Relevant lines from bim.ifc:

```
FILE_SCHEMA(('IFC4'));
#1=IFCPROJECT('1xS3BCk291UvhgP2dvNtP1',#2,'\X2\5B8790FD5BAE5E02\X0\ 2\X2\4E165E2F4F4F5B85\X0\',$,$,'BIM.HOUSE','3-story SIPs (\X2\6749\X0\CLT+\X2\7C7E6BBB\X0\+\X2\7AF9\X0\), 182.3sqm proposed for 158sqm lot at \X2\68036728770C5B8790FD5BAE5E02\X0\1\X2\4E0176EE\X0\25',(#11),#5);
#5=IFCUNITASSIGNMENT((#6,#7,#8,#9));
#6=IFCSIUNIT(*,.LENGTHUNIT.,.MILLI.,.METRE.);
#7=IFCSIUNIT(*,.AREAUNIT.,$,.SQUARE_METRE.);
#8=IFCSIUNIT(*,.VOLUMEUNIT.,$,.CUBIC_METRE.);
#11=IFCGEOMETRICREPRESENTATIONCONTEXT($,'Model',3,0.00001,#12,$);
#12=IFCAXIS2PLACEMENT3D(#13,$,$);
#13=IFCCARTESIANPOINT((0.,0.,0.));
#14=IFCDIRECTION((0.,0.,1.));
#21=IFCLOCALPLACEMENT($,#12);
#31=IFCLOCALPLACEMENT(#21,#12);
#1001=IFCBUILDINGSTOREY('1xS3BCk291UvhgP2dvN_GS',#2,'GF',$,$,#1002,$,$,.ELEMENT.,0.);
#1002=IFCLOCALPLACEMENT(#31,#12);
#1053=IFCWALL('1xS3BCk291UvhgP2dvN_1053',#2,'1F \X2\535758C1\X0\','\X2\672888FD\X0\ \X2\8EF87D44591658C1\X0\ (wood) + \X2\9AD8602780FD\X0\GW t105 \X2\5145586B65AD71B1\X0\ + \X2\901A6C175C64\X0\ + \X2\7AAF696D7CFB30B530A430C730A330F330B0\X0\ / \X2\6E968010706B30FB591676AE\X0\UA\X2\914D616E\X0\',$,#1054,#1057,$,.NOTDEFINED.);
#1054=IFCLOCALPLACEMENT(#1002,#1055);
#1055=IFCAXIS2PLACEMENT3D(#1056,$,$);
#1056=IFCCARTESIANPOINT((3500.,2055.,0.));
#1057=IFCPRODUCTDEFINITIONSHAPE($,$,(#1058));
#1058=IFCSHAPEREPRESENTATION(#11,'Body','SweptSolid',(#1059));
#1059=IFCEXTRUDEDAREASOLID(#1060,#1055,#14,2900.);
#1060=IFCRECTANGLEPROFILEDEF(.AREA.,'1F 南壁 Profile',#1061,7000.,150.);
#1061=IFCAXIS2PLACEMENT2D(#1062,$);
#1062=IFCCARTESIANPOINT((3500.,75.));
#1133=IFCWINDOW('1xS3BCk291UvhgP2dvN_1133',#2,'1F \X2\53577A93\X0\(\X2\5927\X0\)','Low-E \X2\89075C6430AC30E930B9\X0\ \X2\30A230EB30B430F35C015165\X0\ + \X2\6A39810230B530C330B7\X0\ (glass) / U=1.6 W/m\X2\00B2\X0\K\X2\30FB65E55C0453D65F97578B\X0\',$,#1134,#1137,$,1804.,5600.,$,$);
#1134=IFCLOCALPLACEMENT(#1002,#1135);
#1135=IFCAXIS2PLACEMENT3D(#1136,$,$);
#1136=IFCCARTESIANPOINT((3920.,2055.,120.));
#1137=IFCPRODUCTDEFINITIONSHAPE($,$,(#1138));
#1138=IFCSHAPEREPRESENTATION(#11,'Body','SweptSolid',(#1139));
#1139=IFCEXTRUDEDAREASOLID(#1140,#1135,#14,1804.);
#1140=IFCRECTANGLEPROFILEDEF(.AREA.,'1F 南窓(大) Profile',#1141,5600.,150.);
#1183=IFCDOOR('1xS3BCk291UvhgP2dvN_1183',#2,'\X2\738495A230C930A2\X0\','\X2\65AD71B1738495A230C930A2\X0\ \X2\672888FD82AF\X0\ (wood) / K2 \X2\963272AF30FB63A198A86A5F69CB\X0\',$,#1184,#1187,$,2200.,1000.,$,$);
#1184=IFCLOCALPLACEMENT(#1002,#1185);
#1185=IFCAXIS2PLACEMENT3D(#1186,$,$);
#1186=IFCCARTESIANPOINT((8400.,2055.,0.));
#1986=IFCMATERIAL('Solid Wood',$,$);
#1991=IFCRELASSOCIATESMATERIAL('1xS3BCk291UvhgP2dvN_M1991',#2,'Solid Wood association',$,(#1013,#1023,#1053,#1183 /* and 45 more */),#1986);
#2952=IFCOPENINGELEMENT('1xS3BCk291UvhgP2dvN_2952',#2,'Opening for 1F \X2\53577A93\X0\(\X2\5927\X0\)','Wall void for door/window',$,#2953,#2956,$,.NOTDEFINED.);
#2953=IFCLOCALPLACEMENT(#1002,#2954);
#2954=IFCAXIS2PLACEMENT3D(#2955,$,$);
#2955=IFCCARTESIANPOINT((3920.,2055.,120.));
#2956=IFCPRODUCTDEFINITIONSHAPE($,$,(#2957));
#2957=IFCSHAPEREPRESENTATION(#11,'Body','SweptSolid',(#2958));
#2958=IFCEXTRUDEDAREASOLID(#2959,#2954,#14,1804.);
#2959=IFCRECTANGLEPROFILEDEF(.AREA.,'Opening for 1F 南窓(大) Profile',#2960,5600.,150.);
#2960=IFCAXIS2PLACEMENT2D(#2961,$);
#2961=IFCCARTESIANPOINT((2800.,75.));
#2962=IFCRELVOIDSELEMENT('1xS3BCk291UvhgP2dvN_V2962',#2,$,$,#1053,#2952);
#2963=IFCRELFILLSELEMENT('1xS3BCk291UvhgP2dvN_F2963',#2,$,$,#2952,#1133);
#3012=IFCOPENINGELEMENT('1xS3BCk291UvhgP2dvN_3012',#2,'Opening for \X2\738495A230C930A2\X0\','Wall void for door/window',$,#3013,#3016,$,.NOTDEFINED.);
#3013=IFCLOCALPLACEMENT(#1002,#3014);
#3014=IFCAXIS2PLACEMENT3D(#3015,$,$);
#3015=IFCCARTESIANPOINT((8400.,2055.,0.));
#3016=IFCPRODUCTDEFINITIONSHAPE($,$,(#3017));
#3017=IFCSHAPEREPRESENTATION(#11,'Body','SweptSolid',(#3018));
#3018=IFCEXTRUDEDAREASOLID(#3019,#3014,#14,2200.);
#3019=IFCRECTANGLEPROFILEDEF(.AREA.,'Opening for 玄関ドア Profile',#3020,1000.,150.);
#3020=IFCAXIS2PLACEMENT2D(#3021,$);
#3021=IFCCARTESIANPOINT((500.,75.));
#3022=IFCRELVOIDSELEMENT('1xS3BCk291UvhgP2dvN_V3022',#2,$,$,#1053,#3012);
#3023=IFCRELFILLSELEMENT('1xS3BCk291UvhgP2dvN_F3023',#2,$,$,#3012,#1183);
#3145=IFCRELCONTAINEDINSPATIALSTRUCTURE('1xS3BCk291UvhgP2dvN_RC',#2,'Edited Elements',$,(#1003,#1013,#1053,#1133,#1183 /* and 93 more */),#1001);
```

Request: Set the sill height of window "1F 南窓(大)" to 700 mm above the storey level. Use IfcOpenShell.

```python
import numpy as np
import ifcopenshell
import ifcopenshell.api.geometry
import ifcopenshell.geom
import ifcopenshell.util.element
import ifcopenshell.util.placement
import ifcopenshell.util.shape
import ifcopenshell.util.unit

model = ifcopenshell.open("bim.ifc")
unit_scale = ifcopenshell.util.unit.calculate_unit_scale(model)

window = model.by_guid("1xS3BCk291UvhgP2dvN_1133")
opening = window.FillsVoids[0].RelatingOpeningElement
storey = ifcopenshell.util.element.get_container(window, ifc_class="IfcBuildingStorey")
level = ifcopenshell.util.placement.get_local_placement(storey.ObjectPlacement)[2, 3]

# The opening's origin need not be at the sill, so measure its lowest point.
shape = ifcopenshell.geom.create_shape(ifcopenshell.geom.settings(), opening)
bottom = ifcopenshell.util.shape.get_shape_bottom_elevation(shape, shape.geometry) / unit_scale
dz = level + 0.7 / unit_scale - bottom

shift = np.array([0.0, 0.0, dz])
# The window is not placed relative to its opening, so move both.
for product in (opening, window):
    matrix = ifcopenshell.util.placement.get_local_placement(product.ObjectPlacement)
    matrix[:3, 3] += shift
    ifcopenshell.api.geometry.edit_object_placement(model, product=product, matrix=matrix, is_si=False)

print(f"moved by {dz * unit_scale:+.3f} m")

model.write("bim_updated.ifc")
```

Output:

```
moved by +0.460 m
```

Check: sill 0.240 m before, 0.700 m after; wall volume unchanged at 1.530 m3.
